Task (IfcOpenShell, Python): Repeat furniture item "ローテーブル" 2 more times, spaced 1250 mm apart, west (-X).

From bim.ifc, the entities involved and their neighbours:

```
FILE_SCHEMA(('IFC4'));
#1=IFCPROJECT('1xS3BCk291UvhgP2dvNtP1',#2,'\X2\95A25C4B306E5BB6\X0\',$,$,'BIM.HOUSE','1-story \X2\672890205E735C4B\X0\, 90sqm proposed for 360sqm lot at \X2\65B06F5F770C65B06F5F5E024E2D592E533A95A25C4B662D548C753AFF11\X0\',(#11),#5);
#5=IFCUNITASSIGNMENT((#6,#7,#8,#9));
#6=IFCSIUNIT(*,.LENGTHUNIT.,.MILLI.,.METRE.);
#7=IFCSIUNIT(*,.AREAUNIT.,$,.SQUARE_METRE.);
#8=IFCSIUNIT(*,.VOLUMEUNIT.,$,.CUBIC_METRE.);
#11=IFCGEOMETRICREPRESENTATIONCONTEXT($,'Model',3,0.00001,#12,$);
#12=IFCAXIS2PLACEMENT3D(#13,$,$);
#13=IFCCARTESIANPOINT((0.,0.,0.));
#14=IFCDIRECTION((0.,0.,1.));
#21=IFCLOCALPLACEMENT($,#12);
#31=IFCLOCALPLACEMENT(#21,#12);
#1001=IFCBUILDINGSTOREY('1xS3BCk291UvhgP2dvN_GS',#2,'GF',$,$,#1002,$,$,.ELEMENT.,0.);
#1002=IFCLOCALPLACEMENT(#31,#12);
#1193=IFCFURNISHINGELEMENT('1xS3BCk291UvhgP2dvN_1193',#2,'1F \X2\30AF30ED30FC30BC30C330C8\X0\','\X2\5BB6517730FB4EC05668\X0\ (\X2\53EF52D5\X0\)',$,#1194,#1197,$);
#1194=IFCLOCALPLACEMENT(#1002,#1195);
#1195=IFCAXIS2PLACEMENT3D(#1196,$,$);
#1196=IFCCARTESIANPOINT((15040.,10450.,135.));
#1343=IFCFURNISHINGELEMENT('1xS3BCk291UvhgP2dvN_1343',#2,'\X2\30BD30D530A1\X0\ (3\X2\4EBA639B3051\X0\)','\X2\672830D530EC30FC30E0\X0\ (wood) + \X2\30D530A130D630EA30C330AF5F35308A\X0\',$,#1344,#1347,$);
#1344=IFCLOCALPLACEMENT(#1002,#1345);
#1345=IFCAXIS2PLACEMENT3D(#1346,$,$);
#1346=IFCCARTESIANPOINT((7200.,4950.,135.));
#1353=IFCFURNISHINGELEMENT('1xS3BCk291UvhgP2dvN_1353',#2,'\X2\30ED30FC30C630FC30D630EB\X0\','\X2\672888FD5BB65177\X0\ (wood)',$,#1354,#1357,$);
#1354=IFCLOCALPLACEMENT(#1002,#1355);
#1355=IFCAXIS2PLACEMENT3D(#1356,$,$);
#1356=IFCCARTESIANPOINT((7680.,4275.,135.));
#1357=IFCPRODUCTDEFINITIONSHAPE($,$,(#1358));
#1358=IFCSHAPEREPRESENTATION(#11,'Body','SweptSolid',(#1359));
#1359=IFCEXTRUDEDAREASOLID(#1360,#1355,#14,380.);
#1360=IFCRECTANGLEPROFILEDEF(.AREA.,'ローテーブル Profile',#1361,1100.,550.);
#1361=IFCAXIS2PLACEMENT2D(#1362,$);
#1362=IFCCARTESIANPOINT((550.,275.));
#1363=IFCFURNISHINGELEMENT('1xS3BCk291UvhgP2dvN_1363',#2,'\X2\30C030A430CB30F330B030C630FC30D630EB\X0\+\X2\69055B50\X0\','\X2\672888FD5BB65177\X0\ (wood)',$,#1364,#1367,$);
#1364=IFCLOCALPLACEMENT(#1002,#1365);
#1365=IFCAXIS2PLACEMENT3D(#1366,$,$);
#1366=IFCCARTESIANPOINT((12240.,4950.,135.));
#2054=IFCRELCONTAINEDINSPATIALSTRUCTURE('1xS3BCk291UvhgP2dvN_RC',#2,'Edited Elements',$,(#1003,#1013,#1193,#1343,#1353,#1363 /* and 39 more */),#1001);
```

```python
import numpy as np
import ifcopenshell
import ifcopenshell.api.geometry
import ifcopenshell.api.root
import ifcopenshell.util.element
import ifcopenshell.util.placement

model = ifcopenshell.open("bim.ifc")


def reuse_history(source, copy):
    """copy_class also copies each property set's owner history, people and application; keep the originals."""
    for rel in copy.IsDefinedBy:
        if rel.is_a("IfcRelDefinesByProperties") and (history := rel.RelatingPropertyDefinition.OwnerHistory):
            rel.RelatingPropertyDefinition.OwnerHistory = source.OwnerHistory
            ifcopenshell.util.element.remove_deep2(model, history)


source = model.by_guid("1xS3BCk291UvhgP2dvN_1353")
base = ifcopenshell.util.placement.get_local_placement(source.ObjectPlacement)
step = np.array([-1.0, 0.0, 0.0]) * 1250.0

for i in range(1, 3):
    copy = ifcopenshell.api.root.copy_class(model, product=source)
    copy.Representation = ifcopenshell.util.element.copy_deep(
        model, source.Representation, exclude=["IfcGeometricRepresentationContext", "IfcRepresentationMap"]
    )
    reuse_history(source, copy)
    matrix = base.copy()
    matrix[:3, 3] += i * step
    print("added at", matrix[:3, 3].round(3) + 0.0)
    ifcopenshell.api.geometry.edit_object_placement(model, product=copy, matrix=matrix, is_si=False)

model.write("bim_rev.ifc")
```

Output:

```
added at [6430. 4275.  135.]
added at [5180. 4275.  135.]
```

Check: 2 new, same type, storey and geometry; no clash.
